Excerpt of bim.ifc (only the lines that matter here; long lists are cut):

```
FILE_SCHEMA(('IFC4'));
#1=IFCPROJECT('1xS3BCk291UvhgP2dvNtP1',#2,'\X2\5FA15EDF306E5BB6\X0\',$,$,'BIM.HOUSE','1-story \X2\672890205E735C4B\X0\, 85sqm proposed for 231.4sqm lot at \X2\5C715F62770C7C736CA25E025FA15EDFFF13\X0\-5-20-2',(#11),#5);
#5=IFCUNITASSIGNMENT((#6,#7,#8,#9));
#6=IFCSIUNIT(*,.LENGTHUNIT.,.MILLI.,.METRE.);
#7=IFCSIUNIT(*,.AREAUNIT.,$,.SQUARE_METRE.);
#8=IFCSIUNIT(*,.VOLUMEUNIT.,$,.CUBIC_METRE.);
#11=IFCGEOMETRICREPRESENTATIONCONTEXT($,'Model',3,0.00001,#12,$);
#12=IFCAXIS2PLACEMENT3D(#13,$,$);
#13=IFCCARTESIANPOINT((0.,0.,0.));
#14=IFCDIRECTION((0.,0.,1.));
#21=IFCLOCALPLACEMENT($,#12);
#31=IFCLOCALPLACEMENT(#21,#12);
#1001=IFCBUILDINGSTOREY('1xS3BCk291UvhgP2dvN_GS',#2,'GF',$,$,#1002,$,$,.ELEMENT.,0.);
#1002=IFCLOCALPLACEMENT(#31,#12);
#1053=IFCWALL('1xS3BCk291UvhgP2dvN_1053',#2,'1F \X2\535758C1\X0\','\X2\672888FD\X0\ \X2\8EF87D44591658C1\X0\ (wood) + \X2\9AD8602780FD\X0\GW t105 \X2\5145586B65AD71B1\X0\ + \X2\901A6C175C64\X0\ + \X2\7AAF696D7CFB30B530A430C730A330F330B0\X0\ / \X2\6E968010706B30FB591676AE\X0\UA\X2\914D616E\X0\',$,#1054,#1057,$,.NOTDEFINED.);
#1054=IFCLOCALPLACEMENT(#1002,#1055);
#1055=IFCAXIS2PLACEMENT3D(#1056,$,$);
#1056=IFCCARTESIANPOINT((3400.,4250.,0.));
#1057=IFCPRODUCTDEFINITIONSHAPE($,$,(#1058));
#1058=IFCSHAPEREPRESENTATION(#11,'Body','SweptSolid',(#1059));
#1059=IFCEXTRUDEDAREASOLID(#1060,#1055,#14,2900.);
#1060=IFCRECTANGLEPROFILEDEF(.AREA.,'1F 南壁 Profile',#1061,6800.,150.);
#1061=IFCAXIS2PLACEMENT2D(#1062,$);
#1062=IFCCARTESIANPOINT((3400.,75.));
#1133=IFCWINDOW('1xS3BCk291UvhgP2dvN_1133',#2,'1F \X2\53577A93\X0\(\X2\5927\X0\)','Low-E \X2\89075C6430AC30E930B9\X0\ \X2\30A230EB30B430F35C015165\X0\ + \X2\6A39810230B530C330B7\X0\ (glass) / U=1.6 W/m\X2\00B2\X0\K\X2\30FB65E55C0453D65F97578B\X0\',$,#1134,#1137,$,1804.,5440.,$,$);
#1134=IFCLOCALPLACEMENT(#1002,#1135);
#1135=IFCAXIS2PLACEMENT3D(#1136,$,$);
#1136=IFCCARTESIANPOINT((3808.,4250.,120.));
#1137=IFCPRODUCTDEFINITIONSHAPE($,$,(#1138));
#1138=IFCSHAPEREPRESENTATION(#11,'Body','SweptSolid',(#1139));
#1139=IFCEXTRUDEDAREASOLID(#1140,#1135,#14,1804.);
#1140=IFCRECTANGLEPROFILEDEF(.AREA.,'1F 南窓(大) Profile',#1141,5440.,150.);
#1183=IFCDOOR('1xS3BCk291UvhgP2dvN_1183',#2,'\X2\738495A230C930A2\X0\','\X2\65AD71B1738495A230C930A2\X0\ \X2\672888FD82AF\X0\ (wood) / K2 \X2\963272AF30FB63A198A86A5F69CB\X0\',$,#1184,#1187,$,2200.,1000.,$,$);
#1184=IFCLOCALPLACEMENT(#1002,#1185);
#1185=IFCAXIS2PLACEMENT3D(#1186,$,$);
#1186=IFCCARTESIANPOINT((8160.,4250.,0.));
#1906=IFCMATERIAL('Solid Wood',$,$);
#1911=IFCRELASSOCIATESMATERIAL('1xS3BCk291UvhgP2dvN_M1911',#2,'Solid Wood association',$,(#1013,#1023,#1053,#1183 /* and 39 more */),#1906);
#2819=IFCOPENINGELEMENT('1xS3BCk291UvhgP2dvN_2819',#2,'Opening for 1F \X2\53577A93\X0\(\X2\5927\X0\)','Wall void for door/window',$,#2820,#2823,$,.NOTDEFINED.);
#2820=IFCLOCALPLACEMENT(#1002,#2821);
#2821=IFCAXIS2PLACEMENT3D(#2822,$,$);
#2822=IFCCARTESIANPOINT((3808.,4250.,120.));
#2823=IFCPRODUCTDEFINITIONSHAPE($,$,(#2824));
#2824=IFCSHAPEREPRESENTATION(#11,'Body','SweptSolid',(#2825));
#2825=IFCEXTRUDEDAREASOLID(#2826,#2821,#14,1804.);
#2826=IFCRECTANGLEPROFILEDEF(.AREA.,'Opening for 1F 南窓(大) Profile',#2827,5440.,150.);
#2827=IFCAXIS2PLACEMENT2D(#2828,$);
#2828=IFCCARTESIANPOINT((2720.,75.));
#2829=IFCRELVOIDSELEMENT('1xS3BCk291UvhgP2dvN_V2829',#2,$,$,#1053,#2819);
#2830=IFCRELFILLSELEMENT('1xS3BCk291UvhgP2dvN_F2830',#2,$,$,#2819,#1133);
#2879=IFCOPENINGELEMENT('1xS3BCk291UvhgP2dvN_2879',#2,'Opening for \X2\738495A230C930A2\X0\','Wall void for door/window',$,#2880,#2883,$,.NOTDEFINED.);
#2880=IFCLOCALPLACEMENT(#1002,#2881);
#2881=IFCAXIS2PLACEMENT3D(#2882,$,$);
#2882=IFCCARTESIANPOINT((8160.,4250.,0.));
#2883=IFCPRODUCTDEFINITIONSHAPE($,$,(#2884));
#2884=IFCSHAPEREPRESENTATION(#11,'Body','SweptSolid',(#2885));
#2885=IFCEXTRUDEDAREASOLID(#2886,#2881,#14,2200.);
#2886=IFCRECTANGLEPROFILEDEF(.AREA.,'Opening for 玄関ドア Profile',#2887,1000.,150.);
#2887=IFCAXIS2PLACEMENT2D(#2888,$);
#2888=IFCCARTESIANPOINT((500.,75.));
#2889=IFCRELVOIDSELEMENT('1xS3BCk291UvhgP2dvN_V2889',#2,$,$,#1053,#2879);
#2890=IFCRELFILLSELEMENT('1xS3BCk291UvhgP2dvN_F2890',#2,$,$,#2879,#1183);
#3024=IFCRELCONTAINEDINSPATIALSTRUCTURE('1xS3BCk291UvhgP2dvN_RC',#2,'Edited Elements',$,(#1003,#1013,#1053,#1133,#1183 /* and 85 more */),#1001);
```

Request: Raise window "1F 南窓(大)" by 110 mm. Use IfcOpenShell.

```python
import numpy as np
import ifcopenshell
import ifcopenshell.api.geometry
import ifcopenshell.util.placement
import ifcopenshell.util.unit

model = ifcopenshell.open("bim.ifc")
unit_scale = ifcopenshell.util.unit.calculate_unit_scale(model)

window = model.by_guid("1xS3BCk291UvhgP2dvN_1133")
opening = window.FillsVoids[0].RelatingOpeningElement
dz = 110.0

shift = np.array([0.0, 0.0, dz])
# The window is not placed relative to its opening, so move both.
for product in (opening, window):
    matrix = ifcopenshell.util.placement.get_local_placement(product.ObjectPlacement)
    matrix[:3, 3] += shift
    ifcopenshell.api.geometry.edit_object_placement(model, product=product, matrix=matrix, is_si=False)

print(f"moved by {dz * unit_scale:+.3f} m")

model.write("bim-out.ifc")
```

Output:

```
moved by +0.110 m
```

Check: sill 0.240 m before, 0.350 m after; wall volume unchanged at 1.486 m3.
